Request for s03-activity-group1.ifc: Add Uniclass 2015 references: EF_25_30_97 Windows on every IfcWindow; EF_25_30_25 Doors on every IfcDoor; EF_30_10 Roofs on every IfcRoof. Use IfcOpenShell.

First a look at what the model holds.

```python
import ifcopenshell

model = ifcopenshell.open("s03-activity-group1.ifc")
print(model.schema)
print("classifications:", [c.Name for c in model.by_type("IfcClassification")])
for ifc_class in ("IfcDoor", "IfcRoof", "IfcStair", "IfcWall", "IfcWindow"):
    print(ifc_class, len(model.by_type(ifc_class)))
```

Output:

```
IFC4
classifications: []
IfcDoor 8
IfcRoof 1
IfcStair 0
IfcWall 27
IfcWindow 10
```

```python
import ifcopenshell
import ifcopenshell.api.classification

model = ifcopenshell.open("s03-activity-group1.ifc")

system = ifcopenshell.api.classification.add_classification(model, classification="Uniclass 2015")

codes = {
    "IfcWindow": ("EF_25_30_97", "Windows"),
    "IfcDoor": ("EF_25_30_25", "Doors"),
    "IfcRoof": ("EF_30_10", "Roofs"),
}
for ifc_class, (code, name) in codes.items():
    products = model.by_type(ifc_class)
    ifcopenshell.api.classification.add_reference(
        model, products=products, classification=system, identification=code, name=name
    )
    print(code, len(products))

model.write("s03-activity-group1_v2.ifc")
```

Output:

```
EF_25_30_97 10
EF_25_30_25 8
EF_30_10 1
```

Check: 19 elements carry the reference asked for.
